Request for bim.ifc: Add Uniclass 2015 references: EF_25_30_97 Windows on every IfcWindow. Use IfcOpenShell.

First a look at what the model holds.

```python
import ifcopenshell

model = ifcopenshell.open("bim.ifc")
print(model.schema)
print("classifications:", [c.Name for c in model.by_type("IfcClassification")])
for ifc_class in ("IfcDoor", "IfcRoof", "IfcStair", "IfcWall", "IfcWindow"):
    print(ifc_class, len(model.by_type(ifc_class)))
```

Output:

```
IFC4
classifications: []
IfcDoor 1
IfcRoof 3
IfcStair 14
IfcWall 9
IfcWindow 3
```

```python
import ifcopenshell
import ifcopenshell.api.classification

model = ifcopenshell.open("bim.ifc")

system = ifcopenshell.api.classification.add_classification(model, classification="Uniclass 2015")

codes = {
    "IfcWindow": ("EF_25_30_97", "Windows"),
}
for ifc_class, (code, name) in codes.items():
    products = model.by_type(ifc_class)
    ifcopenshell.api.classification.add_reference(
        model, products=products, classification=system, identification=code, name=name
    )
    print(code, len(products))

model.write("bim-out.ifc")
```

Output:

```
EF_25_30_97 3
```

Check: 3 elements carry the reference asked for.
